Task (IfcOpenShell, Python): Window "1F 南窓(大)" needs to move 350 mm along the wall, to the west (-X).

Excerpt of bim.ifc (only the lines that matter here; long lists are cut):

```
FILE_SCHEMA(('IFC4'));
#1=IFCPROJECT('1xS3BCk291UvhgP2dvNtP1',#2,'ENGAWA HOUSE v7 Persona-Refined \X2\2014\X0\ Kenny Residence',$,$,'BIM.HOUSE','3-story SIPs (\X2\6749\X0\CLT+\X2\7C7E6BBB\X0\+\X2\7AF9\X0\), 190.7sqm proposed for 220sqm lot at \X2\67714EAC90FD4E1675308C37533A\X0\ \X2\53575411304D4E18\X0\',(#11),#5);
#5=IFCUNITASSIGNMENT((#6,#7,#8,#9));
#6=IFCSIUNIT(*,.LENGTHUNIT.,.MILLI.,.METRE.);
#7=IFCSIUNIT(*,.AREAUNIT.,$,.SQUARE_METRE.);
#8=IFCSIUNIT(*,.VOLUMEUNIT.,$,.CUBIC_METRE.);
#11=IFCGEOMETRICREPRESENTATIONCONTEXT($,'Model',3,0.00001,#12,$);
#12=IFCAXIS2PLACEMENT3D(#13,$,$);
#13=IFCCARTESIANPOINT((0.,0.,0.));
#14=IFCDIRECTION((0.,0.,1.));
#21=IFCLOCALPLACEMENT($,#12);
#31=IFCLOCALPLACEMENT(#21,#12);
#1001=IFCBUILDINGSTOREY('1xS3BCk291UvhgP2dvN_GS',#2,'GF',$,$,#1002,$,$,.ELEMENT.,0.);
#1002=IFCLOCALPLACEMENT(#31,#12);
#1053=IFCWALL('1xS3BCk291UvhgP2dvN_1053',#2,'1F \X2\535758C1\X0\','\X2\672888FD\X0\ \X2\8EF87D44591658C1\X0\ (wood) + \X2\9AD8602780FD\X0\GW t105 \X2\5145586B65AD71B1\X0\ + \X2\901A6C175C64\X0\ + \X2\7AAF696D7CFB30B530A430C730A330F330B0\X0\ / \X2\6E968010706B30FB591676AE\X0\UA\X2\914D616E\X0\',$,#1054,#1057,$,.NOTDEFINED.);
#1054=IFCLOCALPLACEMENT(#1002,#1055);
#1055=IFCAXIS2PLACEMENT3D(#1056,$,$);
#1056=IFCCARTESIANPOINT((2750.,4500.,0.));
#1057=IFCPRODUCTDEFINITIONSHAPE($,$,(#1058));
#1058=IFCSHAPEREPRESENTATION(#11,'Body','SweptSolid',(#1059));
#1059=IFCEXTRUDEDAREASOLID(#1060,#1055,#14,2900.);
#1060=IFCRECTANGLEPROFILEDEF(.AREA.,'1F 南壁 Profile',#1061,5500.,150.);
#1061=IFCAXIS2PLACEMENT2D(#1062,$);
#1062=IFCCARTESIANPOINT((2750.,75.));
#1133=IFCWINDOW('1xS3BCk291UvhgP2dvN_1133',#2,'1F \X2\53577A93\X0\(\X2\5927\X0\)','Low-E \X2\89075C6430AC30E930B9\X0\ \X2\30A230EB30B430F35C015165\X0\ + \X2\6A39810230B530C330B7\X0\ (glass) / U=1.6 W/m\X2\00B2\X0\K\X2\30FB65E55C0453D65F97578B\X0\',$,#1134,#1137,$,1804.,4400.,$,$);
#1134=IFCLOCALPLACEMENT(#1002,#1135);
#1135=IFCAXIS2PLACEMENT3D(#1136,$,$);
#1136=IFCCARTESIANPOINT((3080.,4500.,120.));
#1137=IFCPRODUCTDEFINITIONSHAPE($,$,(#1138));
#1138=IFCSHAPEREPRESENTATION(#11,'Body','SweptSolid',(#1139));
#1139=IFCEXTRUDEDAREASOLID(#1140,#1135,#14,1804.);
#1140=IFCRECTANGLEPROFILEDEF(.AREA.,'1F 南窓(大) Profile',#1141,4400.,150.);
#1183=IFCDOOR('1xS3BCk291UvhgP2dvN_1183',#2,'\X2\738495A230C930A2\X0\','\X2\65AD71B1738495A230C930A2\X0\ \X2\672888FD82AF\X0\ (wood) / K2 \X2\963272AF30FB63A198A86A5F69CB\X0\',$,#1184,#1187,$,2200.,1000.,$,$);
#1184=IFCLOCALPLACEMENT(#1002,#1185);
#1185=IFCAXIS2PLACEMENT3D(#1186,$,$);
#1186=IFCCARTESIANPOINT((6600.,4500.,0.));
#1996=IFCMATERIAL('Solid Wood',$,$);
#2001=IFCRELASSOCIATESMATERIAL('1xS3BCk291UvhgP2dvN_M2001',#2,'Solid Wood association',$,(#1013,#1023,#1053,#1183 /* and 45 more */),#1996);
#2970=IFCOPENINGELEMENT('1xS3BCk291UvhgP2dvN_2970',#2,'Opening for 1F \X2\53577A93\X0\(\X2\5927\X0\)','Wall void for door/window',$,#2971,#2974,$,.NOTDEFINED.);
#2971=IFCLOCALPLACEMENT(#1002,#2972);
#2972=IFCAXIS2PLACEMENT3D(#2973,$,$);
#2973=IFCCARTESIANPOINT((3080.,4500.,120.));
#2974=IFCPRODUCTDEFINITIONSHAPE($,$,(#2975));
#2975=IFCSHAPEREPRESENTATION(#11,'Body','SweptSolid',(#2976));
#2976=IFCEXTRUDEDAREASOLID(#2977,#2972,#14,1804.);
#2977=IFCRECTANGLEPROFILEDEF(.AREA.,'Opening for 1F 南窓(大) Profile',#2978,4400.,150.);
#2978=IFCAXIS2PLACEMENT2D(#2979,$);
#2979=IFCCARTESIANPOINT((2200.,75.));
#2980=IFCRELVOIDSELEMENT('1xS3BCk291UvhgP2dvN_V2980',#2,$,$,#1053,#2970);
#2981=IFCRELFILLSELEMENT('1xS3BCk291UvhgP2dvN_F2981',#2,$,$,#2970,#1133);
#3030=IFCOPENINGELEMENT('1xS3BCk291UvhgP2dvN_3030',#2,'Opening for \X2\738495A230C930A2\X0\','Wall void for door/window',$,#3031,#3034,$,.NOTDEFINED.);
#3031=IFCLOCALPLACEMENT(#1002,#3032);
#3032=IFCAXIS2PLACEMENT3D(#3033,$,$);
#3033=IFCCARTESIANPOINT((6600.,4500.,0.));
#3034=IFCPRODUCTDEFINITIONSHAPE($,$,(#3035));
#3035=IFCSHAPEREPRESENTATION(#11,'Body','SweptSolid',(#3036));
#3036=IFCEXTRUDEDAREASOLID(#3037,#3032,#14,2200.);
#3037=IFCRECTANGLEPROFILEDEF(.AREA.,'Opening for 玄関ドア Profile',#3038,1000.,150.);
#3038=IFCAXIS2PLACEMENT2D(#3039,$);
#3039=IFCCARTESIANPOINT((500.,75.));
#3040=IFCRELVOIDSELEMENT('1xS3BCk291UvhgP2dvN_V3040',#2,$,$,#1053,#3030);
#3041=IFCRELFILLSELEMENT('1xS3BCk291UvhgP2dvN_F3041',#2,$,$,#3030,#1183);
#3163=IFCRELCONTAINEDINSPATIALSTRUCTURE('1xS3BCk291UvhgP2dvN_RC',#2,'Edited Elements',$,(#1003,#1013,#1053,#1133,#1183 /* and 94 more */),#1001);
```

```python
import ifcopenshell
import ifcopenshell.api.geometry
import ifcopenshell.util.placement
import ifcopenshell.util.unit

model = ifcopenshell.open("bim.ifc")
unit_scale = ifcopenshell.util.unit.calculate_unit_scale(model)

window = model.by_guid("1xS3BCk291UvhgP2dvN_1133")
opening = window.FillsVoids[0].RelatingOpeningElement
wall = opening.VoidsElements[0].RelatingBuildingElement

wall_matrix = ifcopenshell.util.placement.get_local_placement(wall.ObjectPlacement)
shift = wall_matrix[:3, 0] * -0.35 / unit_scale
before = ifcopenshell.util.placement.get_local_placement(window.ObjectPlacement)[:3, 3].copy()

# The window is not placed relative to its opening, so move both.
for product in (opening, window):
    matrix = ifcopenshell.util.placement.get_local_placement(product.ObjectPlacement)
    matrix[:3, 3] += shift
    ifcopenshell.api.geometry.edit_object_placement(model, product=product, matrix=matrix, is_si=False)

after = ifcopenshell.util.placement.get_local_placement(window.ObjectPlacement)[:3, 3]
print("window moved by", (after - before).round(3) + 0.0)

model.write("bim_updated.ifc")
```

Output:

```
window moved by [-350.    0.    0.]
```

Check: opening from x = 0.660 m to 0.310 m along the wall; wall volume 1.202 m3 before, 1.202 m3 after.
